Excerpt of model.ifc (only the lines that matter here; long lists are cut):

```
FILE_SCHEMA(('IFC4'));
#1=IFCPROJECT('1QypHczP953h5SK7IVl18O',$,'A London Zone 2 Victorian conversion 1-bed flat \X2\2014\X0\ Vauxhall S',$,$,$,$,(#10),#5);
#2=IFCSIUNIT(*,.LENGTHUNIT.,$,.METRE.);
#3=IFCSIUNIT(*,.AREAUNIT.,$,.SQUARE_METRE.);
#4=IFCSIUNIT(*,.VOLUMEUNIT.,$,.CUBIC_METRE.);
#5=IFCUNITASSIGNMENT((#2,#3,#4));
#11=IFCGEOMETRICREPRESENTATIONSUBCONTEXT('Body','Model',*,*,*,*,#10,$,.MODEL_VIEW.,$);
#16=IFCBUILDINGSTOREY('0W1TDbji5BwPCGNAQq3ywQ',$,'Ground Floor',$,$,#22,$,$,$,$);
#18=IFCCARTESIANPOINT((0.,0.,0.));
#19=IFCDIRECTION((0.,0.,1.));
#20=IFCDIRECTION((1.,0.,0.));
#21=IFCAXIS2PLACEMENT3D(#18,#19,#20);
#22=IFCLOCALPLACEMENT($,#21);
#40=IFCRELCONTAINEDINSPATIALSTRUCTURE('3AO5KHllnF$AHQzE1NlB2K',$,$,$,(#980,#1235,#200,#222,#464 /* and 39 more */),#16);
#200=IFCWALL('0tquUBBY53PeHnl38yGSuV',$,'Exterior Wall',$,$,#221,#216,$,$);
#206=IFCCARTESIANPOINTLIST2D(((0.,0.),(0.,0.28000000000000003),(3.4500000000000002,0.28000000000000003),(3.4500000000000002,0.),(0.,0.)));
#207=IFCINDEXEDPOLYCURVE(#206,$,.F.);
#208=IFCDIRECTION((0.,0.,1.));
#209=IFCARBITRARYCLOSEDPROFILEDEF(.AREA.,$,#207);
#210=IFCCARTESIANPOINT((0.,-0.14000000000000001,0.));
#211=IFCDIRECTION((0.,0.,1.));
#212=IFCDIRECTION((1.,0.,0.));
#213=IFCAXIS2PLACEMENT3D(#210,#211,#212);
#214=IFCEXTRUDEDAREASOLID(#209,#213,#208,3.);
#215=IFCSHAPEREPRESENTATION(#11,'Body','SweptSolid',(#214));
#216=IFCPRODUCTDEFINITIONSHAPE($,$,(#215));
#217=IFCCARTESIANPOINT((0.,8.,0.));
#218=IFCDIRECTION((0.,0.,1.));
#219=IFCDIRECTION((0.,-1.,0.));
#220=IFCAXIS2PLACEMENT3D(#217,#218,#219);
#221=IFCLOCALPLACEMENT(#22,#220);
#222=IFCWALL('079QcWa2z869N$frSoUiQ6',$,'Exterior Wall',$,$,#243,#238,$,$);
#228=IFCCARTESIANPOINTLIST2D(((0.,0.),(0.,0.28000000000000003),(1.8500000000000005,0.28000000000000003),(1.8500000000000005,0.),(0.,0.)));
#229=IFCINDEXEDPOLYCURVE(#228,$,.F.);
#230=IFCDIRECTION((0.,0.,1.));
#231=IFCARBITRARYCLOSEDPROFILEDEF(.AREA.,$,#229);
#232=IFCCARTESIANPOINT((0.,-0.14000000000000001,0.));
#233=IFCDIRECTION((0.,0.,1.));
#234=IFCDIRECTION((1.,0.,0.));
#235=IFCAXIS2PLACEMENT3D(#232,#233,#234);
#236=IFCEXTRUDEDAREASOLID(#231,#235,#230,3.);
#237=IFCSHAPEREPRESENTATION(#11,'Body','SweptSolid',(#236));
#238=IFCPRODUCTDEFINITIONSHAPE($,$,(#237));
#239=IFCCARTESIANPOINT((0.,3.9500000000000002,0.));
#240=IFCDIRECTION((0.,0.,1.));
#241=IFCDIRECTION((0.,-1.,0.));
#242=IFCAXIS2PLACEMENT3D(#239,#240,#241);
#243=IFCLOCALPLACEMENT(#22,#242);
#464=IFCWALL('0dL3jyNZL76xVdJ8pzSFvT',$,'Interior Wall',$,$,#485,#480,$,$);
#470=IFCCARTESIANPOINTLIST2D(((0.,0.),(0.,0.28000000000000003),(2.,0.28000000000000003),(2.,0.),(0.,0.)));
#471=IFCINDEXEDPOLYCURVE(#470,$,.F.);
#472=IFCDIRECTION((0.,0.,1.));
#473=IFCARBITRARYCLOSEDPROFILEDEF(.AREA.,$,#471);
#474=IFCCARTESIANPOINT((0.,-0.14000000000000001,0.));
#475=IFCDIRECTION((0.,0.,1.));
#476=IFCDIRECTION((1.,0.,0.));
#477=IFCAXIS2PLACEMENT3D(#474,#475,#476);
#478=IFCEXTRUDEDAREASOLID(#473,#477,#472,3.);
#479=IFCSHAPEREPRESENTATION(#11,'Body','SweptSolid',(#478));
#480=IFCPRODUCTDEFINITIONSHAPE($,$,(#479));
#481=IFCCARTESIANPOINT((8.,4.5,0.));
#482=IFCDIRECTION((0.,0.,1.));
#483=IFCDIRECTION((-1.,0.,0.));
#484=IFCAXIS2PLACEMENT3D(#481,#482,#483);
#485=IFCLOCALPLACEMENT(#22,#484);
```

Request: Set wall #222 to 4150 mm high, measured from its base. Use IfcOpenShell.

```python
import ifcopenshell
import ifcopenshell.geom
import ifcopenshell.util.representation
import ifcopenshell.util.shape
import ifcopenshell.util.unit

model = ifcopenshell.open("model.ifc")
unit_scale = ifcopenshell.util.unit.calculate_unit_scale(model)
settings = ifcopenshell.geom.settings()


def volume(element):
    """Net volume in cubic metres, openings subtracted."""
    shape = ifcopenshell.geom.create_shape(settings, element)
    return ifcopenshell.util.shape.get_volume(shape.geometry)


wall = model.by_guid("079QcWa2z869N$frSoUiQ6")
before = volume(wall)

body = ifcopenshell.util.representation.get_representation(wall, "Model", "Body")
solid = body.Items[0]
old_height = solid.Depth
solid.Depth = 4.15 / unit_scale
after = volume(wall)

print(f"height {old_height:g} -> {solid.Depth:g}, volume {before:.3f} -> {after:.3f} m3")

model.write("model_edited.ifc")
```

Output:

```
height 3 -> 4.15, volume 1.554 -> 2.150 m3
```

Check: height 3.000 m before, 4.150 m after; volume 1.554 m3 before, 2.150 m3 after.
